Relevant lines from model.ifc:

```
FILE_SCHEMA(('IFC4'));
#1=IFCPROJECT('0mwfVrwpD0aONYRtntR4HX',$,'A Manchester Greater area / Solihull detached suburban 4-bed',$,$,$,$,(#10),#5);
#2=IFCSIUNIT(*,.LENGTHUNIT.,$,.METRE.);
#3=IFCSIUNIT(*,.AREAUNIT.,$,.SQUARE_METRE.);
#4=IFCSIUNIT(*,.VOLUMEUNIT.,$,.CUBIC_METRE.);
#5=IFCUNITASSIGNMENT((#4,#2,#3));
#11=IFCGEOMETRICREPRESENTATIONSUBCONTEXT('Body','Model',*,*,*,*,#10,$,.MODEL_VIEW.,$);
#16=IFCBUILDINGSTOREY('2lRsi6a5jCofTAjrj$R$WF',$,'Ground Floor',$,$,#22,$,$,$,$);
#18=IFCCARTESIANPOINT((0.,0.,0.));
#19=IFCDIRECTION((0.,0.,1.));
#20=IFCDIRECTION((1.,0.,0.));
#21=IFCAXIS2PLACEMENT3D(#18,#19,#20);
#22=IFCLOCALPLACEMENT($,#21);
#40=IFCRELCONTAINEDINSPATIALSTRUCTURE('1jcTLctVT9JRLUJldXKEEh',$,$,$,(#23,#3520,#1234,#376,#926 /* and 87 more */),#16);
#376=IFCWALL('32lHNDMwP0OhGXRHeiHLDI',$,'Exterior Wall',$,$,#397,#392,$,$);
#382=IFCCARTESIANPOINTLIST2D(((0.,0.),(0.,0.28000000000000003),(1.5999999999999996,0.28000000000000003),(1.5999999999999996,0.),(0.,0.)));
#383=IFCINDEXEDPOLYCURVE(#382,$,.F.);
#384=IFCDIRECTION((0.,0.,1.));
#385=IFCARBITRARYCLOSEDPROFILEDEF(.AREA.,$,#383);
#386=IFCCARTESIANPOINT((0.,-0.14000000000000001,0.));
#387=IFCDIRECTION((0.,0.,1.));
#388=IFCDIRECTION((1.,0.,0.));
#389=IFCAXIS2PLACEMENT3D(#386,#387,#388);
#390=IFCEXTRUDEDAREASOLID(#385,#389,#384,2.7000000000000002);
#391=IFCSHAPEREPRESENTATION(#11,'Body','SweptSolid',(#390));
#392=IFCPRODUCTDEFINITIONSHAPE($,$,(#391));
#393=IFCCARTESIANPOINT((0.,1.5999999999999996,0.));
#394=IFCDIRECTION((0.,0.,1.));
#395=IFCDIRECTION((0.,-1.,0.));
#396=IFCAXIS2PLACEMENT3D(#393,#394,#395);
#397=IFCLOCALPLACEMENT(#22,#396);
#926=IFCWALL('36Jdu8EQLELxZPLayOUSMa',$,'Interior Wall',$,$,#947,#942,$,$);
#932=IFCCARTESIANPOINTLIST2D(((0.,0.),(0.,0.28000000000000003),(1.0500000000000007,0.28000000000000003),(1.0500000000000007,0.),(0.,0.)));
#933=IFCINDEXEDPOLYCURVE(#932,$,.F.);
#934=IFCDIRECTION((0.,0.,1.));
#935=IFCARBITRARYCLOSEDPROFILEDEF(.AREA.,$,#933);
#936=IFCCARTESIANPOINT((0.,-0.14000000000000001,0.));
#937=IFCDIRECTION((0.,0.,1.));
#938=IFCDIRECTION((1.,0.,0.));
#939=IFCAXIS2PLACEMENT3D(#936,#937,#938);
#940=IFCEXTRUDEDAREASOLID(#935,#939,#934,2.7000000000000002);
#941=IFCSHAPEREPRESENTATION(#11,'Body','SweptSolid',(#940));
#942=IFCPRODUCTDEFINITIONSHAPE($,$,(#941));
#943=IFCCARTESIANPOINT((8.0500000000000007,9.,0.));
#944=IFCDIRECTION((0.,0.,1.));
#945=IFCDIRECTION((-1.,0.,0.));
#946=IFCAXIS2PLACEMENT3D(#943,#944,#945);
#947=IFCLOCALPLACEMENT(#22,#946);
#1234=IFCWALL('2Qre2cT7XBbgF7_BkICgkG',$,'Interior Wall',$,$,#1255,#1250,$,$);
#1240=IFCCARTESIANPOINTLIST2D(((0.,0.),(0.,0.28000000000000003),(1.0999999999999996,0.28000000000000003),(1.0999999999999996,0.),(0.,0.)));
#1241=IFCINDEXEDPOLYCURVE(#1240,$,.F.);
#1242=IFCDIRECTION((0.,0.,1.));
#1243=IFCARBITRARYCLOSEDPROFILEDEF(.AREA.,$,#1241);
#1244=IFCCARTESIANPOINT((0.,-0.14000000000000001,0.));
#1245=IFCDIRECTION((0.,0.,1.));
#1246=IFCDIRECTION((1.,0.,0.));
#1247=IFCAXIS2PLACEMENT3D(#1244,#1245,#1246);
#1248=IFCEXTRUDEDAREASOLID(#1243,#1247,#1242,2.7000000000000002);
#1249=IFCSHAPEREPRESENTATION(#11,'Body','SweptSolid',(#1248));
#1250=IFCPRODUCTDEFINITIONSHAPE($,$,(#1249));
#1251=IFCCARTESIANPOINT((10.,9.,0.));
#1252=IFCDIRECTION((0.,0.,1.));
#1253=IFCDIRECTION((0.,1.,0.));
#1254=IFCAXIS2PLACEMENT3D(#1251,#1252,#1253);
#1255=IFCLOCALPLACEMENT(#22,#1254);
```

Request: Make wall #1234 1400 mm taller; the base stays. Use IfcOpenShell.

```python
import ifcopenshell
import ifcopenshell.geom
import ifcopenshell.util.representation
import ifcopenshell.util.shape

model = ifcopenshell.open("model.ifc")
settings = ifcopenshell.geom.settings()


def volume(element):
    """Net volume in cubic metres, openings subtracted."""
    shape = ifcopenshell.geom.create_shape(settings, element)
    return ifcopenshell.util.shape.get_volume(shape.geometry)


wall = model.by_id(1234)
before = volume(wall)

body = ifcopenshell.util.representation.get_representation(wall, "Model", "Body")
solid = body.Items[0]
old_height = solid.Depth
solid.Depth += 1.4
after = volume(wall)

print(f"height {old_height:g} -> {solid.Depth:g}, volume {before:.3f} -> {after:.3f} m3")

model.write("model_v2.ifc")
```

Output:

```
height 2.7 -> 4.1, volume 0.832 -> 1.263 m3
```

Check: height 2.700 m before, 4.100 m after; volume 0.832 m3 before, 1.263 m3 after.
